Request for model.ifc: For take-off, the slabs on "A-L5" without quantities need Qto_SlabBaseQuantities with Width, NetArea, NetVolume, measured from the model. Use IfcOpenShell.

First a look at what the model holds.

```python
import ifcopenshell
import ifcopenshell.util.element
import ifcopenshell.util.unit

model = ifcopenshell.open("model.ifc")
print(model.schema)
for unit_type in ("LENGTHUNIT", "AREAUNIT", "VOLUMEUNIT"):
    print(unit_type, ifcopenshell.util.unit.calculate_unit_scale(model, unit_type))
storey = next(s for s in model.by_type("IfcBuildingStorey") if s.Name == "A-L5")
slabs = [e for e in ifcopenshell.util.element.get_decomposition(storey) if e.is_a("IfcSlab")]
for e in sorted(slabs, key=lambda e: e.id()):
    print(e.id(), e.is_a(), e.Name, list(ifcopenshell.util.element.get_psets(e, qtos_only=True)), sep=" | ")
```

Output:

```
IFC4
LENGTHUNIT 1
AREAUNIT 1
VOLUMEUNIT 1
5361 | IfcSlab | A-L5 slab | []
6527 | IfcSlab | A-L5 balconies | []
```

```python
import ifcopenshell
import ifcopenshell.api.pset
import ifcopenshell.geom
import ifcopenshell.util.element
import ifcopenshell.util.shape
import ifcopenshell.util.unit

model = ifcopenshell.open("model.ifc")
unit_scale = ifcopenshell.util.unit.calculate_unit_scale(model)
area_scale = ifcopenshell.util.unit.calculate_unit_scale(model, "AREAUNIT")
volume_scale = ifcopenshell.util.unit.calculate_unit_scale(model, "VOLUMEUNIT")
settings = ifcopenshell.geom.settings()

storey = next(s for s in model.by_type("IfcBuildingStorey") if s.Name == "A-L5")
slabs = [e for e in ifcopenshell.util.element.get_decomposition(storey) if e.is_a("IfcSlab")]

for e in sorted(slabs, key=lambda e: e.id()):
    if ifcopenshell.util.element.get_psets(e, qtos_only=True, should_inherit=False):
        continue
    # Geometry comes back in metres, in the element's own axes.
    shape = ifcopenshell.geom.create_shape(settings, e)
    values = {
        "Width": ifcopenshell.util.shape.get_z(shape.geometry) / unit_scale,
        "NetArea": ifcopenshell.util.shape.get_footprint_area(shape.geometry) / area_scale,
        "NetVolume": ifcopenshell.util.shape.get_volume(shape.geometry) / volume_scale,
    }
    qto = ifcopenshell.api.pset.add_qto(model, product=e, name="Qto_SlabBaseQuantities")
    ifcopenshell.api.pset.edit_qto(model, qto=qto, properties=values)
    print(e.id(), {k: round(v, 3) for k, v in values.items()})

model.write("model_v2.ifc")
```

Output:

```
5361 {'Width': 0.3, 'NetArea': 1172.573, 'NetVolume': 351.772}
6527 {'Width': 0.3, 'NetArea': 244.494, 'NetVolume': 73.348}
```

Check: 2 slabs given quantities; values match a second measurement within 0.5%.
